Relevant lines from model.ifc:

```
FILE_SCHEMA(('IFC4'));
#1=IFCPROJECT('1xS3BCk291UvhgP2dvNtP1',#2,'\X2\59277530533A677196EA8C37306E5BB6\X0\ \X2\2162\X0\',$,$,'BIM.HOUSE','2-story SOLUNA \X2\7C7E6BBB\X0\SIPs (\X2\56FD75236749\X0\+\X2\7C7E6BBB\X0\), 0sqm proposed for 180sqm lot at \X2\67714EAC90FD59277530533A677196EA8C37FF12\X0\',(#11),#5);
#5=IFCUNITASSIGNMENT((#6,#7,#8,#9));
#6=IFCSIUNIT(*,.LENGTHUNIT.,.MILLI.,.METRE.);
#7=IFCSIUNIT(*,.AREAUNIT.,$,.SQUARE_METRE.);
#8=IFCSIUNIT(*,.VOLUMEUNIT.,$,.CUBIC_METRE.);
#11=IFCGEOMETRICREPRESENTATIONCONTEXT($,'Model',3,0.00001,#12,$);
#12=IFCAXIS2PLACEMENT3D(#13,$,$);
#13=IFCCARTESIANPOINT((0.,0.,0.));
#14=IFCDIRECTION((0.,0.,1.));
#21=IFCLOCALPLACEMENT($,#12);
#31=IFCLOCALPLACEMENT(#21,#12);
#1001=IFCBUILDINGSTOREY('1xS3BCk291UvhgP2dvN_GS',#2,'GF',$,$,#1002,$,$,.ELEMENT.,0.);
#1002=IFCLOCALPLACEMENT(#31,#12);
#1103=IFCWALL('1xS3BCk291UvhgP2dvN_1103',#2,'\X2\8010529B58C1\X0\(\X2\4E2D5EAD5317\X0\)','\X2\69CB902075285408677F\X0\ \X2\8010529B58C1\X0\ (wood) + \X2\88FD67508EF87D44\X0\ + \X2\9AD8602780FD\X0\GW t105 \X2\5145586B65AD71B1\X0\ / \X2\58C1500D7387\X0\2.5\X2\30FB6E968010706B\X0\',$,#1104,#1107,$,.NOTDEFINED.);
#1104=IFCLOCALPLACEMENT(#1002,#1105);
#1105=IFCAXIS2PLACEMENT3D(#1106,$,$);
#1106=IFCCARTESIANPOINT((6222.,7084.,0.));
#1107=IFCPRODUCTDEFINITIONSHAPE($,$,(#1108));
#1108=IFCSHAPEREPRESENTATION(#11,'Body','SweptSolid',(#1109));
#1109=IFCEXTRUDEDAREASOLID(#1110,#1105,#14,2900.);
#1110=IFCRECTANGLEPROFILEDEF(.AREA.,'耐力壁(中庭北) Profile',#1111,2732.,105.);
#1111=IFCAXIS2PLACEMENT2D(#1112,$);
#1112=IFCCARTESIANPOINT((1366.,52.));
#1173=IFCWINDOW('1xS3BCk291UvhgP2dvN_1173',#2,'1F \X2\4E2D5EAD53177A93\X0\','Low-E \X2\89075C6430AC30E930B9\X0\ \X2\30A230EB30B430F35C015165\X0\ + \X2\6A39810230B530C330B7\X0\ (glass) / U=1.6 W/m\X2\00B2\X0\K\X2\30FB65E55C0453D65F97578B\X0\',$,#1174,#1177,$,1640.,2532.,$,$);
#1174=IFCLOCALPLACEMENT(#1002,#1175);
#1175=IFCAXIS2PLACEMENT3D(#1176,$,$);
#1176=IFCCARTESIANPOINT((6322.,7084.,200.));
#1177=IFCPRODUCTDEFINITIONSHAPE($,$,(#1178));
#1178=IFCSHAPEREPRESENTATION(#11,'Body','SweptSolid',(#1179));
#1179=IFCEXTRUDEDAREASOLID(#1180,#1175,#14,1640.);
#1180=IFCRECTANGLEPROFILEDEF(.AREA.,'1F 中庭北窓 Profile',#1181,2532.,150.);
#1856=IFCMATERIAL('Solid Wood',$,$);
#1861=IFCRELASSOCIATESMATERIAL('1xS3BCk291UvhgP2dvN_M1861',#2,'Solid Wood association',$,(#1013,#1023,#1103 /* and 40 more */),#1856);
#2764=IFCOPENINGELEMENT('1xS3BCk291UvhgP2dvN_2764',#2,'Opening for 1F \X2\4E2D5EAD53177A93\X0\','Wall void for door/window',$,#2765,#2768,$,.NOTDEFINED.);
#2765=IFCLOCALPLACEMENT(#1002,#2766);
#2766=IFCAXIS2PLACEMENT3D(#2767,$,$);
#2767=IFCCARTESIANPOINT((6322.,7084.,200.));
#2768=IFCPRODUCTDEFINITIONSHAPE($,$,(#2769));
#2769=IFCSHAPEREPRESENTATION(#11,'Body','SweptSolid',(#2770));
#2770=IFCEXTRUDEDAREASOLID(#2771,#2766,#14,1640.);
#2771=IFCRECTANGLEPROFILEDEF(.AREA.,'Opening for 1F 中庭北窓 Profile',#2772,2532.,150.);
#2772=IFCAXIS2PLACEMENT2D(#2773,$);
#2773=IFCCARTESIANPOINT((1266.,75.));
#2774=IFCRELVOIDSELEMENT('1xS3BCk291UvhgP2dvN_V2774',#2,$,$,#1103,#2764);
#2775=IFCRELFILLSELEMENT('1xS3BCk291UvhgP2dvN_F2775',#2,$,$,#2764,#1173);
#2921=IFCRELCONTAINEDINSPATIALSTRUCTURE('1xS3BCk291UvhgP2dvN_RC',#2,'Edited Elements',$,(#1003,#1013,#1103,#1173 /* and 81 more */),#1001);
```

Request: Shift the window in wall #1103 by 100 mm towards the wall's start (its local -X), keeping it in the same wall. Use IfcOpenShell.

```python
import ifcopenshell
import ifcopenshell.api.geometry
import ifcopenshell.util.placement

model = ifcopenshell.open("model.ifc")

window = model.by_guid("1xS3BCk291UvhgP2dvN_1173")
opening = window.FillsVoids[0].RelatingOpeningElement
wall = opening.VoidsElements[0].RelatingBuildingElement

wall_matrix = ifcopenshell.util.placement.get_local_placement(wall.ObjectPlacement)
shift = wall_matrix[:3, 0] * -100.0
before = ifcopenshell.util.placement.get_local_placement(window.ObjectPlacement)[:3, 3].copy()

# The window is not placed relative to its opening, so move both.
for product in (opening, window):
    matrix = ifcopenshell.util.placement.get_local_placement(product.ObjectPlacement)
    matrix[:3, 3] += shift
    ifcopenshell.api.geometry.edit_object_placement(model, product=product, matrix=matrix, is_si=False)

after = ifcopenshell.util.placement.get_local_placement(window.ObjectPlacement)[:3, 3]
print("window moved by", (after - before).round(3) + 0.0)

model.write("model_rev.ifc")
```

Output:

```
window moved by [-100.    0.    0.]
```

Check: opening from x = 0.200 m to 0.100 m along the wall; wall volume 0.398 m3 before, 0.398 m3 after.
